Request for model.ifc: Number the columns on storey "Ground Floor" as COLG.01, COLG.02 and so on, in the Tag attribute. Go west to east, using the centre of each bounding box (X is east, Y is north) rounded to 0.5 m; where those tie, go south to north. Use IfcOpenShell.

First a look at what the model holds.

```python
import ifcopenshell
import ifcopenshell.util.element
import ifcopenshell.util.placement

model = ifcopenshell.open("model.ifc")
print(model.schema)
storey = next(s for s in model.by_type("IfcBuildingStorey") if s.Name == "Ground Floor")
columns = [e for e in ifcopenshell.util.element.get_decomposition(storey) if e.is_a("IfcColumn")]
for e in sorted(columns, key=lambda e: e.id()):
    origin = ifcopenshell.util.placement.get_local_placement(e.ObjectPlacement)[:3, 3]
    print(e.id(), e.Tag, e.Name, origin.round(2) + 0.0, sep=" | ")
```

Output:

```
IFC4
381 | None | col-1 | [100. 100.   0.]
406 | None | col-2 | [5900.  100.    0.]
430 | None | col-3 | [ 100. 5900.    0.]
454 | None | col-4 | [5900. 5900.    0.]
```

```python
import ifcopenshell
import ifcopenshell.geom
import ifcopenshell.util.element
import ifcopenshell.util.shape

model = ifcopenshell.open("model.ifc")
settings = ifcopenshell.geom.settings()
settings.set("use-world-coords", True)


def centre(element):
    shape = ifcopenshell.geom.create_shape(settings, element)
    return ifcopenshell.util.shape.get_bbox_centroid(shape.geometry)


storey = next(s for s in model.by_type("IfcBuildingStorey") if s.Name == "Ground Floor")
columns = [e for e in ifcopenshell.util.element.get_decomposition(storey) if e.is_a("IfcColumn")]

# Insertion points can sit at a corner or the storey origin, so sort by the geometry (in metres).
centres = {e: centre(e) for e in columns}
columns.sort(key=lambda e: (round(centres[e][0] / 0.5), centres[e][1]))

for i, e in enumerate(columns, start=1):
    number = f"COLG.{i:02d}"
    e.Tag = number
    print(e.id(), number)

model.write("model_v2.ifc")
```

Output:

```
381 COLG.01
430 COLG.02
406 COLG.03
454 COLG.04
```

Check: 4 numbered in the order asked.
